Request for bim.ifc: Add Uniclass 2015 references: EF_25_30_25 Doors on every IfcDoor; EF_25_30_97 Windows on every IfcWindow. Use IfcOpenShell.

First a look at what the model holds.

```python
import ifcopenshell

model = ifcopenshell.open("bim.ifc")
print(model.schema)
print("classifications:", [c.Name for c in model.by_type("IfcClassification")])
for ifc_class in ("IfcDoor", "IfcRoof", "IfcStair", "IfcWall", "IfcWindow"):
    print(ifc_class, len(model.by_type(ifc_class)))
```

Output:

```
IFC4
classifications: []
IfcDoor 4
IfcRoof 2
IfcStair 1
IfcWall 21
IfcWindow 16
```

```python
import ifcopenshell
import ifcopenshell.api.classification

model = ifcopenshell.open("bim.ifc")

system = ifcopenshell.api.classification.add_classification(model, classification="Uniclass 2015")

codes = {
    "IfcDoor": ("EF_25_30_25", "Doors"),
    "IfcWindow": ("EF_25_30_97", "Windows"),
}
for ifc_class, (code, name) in codes.items():
    products = model.by_type(ifc_class)
    ifcopenshell.api.classification.add_reference(
        model, products=products, classification=system, identification=code, name=name
    )
    print(code, len(products))

model.write("bim-out.ifc")
```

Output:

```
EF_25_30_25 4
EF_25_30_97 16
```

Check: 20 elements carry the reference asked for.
